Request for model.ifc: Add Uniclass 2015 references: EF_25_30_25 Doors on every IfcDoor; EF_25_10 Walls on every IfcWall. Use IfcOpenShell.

First a look at what the model holds.

```python
import ifcopenshell

model = ifcopenshell.open("model.ifc")
print(model.schema)
print("classifications:", [c.Name for c in model.by_type("IfcClassification")])
for ifc_class in ("IfcDoor", "IfcRoof", "IfcStair", "IfcWall", "IfcWindow"):
    print(ifc_class, len(model.by_type(ifc_class)))
```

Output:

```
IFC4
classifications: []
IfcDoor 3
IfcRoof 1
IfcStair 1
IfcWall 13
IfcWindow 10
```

```python
import ifcopenshell
import ifcopenshell.api.classification

model = ifcopenshell.open("model.ifc")

system = ifcopenshell.api.classification.add_classification(model, classification="Uniclass 2015")

codes = {
    "IfcDoor": ("EF_25_30_25", "Doors"),
    "IfcWall": ("EF_25_10", "Walls"),
}
for ifc_class, (code, name) in codes.items():
    products = model.by_type(ifc_class)
    ifcopenshell.api.classification.add_reference(
        model, products=products, classification=system, identification=code, name=name
    )
    print(code, len(products))

model.write("model_rev.ifc")
```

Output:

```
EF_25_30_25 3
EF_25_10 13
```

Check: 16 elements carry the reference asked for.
